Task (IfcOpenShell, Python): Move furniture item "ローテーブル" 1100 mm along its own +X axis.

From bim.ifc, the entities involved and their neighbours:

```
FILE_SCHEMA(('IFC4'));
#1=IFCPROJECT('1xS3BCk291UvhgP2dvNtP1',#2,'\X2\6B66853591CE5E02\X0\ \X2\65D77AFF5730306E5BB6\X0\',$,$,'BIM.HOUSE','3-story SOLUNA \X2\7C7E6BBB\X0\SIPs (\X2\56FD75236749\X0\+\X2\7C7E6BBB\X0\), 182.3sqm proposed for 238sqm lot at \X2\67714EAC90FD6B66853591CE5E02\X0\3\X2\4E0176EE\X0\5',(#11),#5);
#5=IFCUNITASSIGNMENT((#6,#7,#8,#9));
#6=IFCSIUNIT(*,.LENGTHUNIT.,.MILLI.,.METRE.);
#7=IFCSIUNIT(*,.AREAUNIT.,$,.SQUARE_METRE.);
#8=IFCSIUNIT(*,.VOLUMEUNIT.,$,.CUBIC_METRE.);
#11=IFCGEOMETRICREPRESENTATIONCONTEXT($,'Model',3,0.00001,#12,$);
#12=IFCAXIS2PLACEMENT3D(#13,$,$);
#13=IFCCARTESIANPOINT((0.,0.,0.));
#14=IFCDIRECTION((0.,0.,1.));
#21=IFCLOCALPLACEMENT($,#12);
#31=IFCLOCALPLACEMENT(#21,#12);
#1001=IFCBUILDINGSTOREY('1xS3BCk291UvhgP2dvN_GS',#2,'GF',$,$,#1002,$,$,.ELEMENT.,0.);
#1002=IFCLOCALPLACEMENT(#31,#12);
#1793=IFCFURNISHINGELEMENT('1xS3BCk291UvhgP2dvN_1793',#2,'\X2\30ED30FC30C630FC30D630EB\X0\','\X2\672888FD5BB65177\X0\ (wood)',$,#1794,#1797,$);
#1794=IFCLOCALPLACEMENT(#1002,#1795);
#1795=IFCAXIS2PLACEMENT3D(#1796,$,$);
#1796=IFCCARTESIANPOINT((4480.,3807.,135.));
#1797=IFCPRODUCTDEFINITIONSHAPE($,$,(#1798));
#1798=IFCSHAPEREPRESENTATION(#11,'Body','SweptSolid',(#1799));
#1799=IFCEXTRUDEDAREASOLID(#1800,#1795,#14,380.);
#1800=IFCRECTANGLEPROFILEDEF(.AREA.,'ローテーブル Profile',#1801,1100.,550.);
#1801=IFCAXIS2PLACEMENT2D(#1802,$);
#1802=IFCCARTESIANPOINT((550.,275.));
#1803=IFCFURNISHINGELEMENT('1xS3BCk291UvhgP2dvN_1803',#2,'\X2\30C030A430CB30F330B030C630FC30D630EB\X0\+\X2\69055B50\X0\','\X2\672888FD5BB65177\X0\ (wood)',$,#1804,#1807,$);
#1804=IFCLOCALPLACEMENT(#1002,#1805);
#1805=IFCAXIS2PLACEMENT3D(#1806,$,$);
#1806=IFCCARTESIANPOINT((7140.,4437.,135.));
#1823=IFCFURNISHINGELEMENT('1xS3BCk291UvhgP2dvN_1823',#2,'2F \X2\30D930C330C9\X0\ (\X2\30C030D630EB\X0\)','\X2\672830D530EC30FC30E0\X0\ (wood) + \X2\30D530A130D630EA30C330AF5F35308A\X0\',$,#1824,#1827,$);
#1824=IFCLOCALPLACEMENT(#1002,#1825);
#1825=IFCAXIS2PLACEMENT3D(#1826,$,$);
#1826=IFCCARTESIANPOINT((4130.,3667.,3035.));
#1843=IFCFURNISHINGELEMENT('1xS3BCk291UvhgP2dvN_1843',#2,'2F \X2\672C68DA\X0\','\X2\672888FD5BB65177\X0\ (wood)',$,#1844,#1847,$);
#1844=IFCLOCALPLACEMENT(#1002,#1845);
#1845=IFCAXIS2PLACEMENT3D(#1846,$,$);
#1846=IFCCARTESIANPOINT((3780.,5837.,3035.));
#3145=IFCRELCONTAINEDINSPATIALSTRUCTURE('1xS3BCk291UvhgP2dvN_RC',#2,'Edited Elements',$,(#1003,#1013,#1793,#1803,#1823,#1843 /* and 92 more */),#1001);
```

```python
import ifcopenshell
import ifcopenshell.api.geometry
import ifcopenshell.util.placement

model = ifcopenshell.open("bim.ifc")

item = model.by_guid("1xS3BCk291UvhgP2dvN_1793")
matrix = ifcopenshell.util.placement.get_local_placement(item.ObjectPlacement)
matrix[:3, 3] += matrix[:3, 0] * 1100.0
ifcopenshell.api.geometry.edit_object_placement(model, product=item, matrix=matrix, is_si=False)

print(ifcopenshell.util.placement.get_local_placement(item.ObjectPlacement).round(3) + 0.0)

model.write("bim_edited.ifc")
```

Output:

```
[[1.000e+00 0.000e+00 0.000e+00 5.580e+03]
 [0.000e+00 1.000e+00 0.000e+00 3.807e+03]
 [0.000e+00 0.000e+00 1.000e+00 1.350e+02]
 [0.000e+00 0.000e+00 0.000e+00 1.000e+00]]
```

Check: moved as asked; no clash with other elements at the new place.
